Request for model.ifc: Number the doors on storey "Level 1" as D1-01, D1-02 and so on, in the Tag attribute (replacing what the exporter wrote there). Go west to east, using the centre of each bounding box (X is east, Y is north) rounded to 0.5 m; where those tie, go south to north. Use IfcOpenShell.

First a look at what the model holds.

```python
import ifcopenshell
import ifcopenshell.util.element
import ifcopenshell.util.placement

model = ifcopenshell.open("model.ifc")
print(model.schema)
storey = next(s for s in model.by_type("IfcBuildingStorey") if s.Name == "Level 1")
doors = [e for e in ifcopenshell.util.element.get_decomposition(storey) if e.is_a("IfcDoor")]
for e in sorted(doors, key=lambda e: e.id()):
    origin = ifcopenshell.util.placement.get_local_placement(e.ObjectPlacement)[:3, 3]
    print(e.id(), e.Tag, e.Name, origin.round(2) + 0.0, sep=" | ")
```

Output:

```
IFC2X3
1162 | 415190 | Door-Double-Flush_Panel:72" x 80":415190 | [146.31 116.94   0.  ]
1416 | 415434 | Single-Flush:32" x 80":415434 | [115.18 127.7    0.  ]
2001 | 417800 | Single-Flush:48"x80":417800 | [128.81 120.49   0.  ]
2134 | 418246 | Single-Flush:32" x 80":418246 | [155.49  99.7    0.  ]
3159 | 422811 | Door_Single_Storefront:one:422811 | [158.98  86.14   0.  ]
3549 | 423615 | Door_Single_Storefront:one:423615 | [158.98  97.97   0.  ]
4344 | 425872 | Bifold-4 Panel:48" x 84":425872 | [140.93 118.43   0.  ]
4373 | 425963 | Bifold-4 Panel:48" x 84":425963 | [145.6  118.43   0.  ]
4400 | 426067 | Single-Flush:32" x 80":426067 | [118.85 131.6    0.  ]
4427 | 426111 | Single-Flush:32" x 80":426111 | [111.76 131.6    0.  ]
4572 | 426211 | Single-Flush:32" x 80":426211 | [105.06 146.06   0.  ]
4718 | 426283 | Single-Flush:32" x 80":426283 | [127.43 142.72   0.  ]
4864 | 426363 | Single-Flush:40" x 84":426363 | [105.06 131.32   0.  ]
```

```python
import ifcopenshell
import ifcopenshell.geom
import ifcopenshell.util.element
import ifcopenshell.util.shape

model = ifcopenshell.open("model.ifc")
settings = ifcopenshell.geom.settings()
settings.set("use-world-coords", True)


def centre(element):
    shape = ifcopenshell.geom.create_shape(settings, element)
    return ifcopenshell.util.shape.get_bbox_centroid(shape.geometry)


storey = next(s for s in model.by_type("IfcBuildingStorey") if s.Name == "Level 1")
doors = [e for e in ifcopenshell.util.element.get_decomposition(storey) if e.is_a("IfcDoor")]

# Insertion points can sit at a corner or the storey origin, so sort by the geometry (in metres).
centres = {e: centre(e) for e in doors}
doors.sort(key=lambda e: (round(centres[e][0] / 0.5), centres[e][1]))

for i, e in enumerate(doors, start=1):
    number = f"D1-{i:02d}"
    e.Tag = number
    print(e.id(), number)

model.write("model_rev.ifc")
```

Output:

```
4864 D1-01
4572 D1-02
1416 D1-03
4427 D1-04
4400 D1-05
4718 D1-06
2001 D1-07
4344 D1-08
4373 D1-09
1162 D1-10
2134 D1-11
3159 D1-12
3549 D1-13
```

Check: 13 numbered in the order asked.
